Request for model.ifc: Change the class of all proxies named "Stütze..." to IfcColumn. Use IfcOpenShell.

First a look at what the model holds.

```python
import re

import ifcopenshell

model = ifcopenshell.open("model.ifc")
print(model.schema)
seen = {}
for e in model.by_type("IfcBuildingElementProxy"):
    name = re.sub(r":\d+(:\d+)?$", "", e.Name or "")  # drop the element id that some exporters append
    seen[name] = seen.get(name, 0) + 1
for name, count in sorted(seen.items()):
    print(count, "x", name)
```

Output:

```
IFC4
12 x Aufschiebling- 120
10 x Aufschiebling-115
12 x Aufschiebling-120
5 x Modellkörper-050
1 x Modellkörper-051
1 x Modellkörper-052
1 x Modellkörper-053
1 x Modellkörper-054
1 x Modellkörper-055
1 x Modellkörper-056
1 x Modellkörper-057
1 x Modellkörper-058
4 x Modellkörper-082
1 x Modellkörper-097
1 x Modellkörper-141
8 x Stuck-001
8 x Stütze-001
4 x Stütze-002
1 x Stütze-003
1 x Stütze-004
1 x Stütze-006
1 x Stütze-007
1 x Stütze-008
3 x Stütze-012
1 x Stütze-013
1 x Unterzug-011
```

```python
import ifcopenshell
import ifcopenshell.api.root

model = ifcopenshell.open("model.ifc")

proxies = [e.id() for e in model.by_type("IfcBuildingElementProxy") if (e.Name or "").startswith("Stütze")]
for step_id in proxies:
    proxy = model.by_id(step_id)
    # Reclassifying a typed element also reclassifies its type and the type's other occurrences.
    if proxy.is_a("IfcBuildingElementProxy"):
        ifcopenshell.api.root.reassign_class(model, product=proxy, ifc_class="IfcColumn")

print(sum(model.by_id(i).is_a("IfcColumn") for i in proxies), "reclassified")

model.write("model-out.ifc")
```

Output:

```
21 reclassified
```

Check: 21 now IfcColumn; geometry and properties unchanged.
